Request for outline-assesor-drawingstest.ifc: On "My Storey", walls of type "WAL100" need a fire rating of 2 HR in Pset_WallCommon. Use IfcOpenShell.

First a look at what the model holds.

```python
import ifcopenshell
import ifcopenshell.util.element

model = ifcopenshell.open("outline-assesor-drawingstest.ifc")
print(model.schema)
storey = next(s for s in model.by_type("IfcBuildingStorey") if s.Name == "My Storey")
walls = [e for e in ifcopenshell.util.element.get_decomposition(storey) if e.is_a("IfcWall")]
seen = {}
for e in walls:
    element_type = ifcopenshell.util.element.get_type(e)
    key = (element_type.Name if element_type != e and element_type else None, ifcopenshell.util.element.get_pset(e, "Pset_WallCommon", "FireRating"))
    seen[key] = seen.get(key, 0) + 1
for (name, value), count in sorted(seen.items(), key=str):
    print(count, "x", name, "|", value)
```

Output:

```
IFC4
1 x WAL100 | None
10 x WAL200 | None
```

```python
import ifcopenshell
import ifcopenshell.api.pset
import ifcopenshell.util.element

model = ifcopenshell.open("outline-assesor-drawingstest.ifc")

storey = next(s for s in model.by_type("IfcBuildingStorey") if s.Name == "My Storey")
walls = [e for e in ifcopenshell.util.element.get_decomposition(storey) if e.is_a("IfcWall")]

count = 0
for e in walls:
    element_type = ifcopenshell.util.element.get_type(e)
    if element_type in (None, e) or element_type.Name != "WAL100":
        continue
    # add_pset returns the element's existing set when there is one.
    pset = ifcopenshell.api.pset.add_pset(model, product=e, name="Pset_WallCommon")
    ifcopenshell.api.pset.edit_pset(model, pset=pset, properties={"FireRating": "2 HR"})
    count += 1

print(count, "walls updated")

model.write("outline-assesor-drawingstest-out.ifc")
```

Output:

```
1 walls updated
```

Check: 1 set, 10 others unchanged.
